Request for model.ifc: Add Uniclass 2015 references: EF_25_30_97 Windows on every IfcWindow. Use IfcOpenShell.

First a look at what the model holds.

```python
import ifcopenshell

model = ifcopenshell.open("model.ifc")
print(model.schema)
print("classifications:", [c.Name for c in model.by_type("IfcClassification")])
for ifc_class in ("IfcDoor", "IfcRoof", "IfcStair", "IfcWall", "IfcWindow"):
    print(ifc_class, len(model.by_type(ifc_class)))
```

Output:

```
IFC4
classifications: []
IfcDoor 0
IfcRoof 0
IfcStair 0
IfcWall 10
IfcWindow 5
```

```python
import ifcopenshell
import ifcopenshell.api.classification

model = ifcopenshell.open("model.ifc")

system = ifcopenshell.api.classification.add_classification(model, classification="Uniclass 2015")

codes = {
    "IfcWindow": ("EF_25_30_97", "Windows"),
}
for ifc_class, (code, name) in codes.items():
    products = model.by_type(ifc_class)
    ifcopenshell.api.classification.add_reference(
        model, products=products, classification=system, identification=code, name=name
    )
    print(code, len(products))

model.write("model_edited.ifc")
```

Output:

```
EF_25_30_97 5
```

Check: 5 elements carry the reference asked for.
